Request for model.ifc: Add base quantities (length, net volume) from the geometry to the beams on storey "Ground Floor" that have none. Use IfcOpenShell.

First a look at what the model holds.

```python
import ifcopenshell
import ifcopenshell.util.element
import ifcopenshell.util.unit

model = ifcopenshell.open("model.ifc")
print(model.schema)
for unit_type in ("LENGTHUNIT", "AREAUNIT", "VOLUMEUNIT"):
    print(unit_type, ifcopenshell.util.unit.calculate_unit_scale(model, unit_type))
storey = next(s for s in model.by_type("IfcBuildingStorey") if s.Name == "Ground Floor")
beams = [e for e in ifcopenshell.util.element.get_decomposition(storey) if e.is_a("IfcBeam")]
for e in sorted(beams, key=lambda e: e.id()):
    print(e.id(), e.is_a(), e.Name, list(ifcopenshell.util.element.get_psets(e, qtos_only=True)), sep=" | ")
```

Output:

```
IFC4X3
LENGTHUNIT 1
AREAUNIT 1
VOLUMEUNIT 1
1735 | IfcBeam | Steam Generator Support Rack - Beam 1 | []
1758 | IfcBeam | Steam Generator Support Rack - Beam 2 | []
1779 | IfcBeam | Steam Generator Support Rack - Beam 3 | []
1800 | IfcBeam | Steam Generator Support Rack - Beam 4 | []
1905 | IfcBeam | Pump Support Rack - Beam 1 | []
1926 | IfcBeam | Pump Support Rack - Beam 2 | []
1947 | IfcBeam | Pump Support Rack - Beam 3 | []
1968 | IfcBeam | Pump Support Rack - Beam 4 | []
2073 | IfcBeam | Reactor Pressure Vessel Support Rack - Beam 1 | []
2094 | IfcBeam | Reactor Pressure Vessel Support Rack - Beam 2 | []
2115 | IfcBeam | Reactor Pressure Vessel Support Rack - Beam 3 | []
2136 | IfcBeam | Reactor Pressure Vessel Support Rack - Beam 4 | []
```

```python
import ifcopenshell
import ifcopenshell.api.pset
import ifcopenshell.geom
import ifcopenshell.util.element
import ifcopenshell.util.shape
import ifcopenshell.util.unit

model = ifcopenshell.open("model.ifc")
unit_scale = ifcopenshell.util.unit.calculate_unit_scale(model)
volume_scale = ifcopenshell.util.unit.calculate_unit_scale(model, "VOLUMEUNIT")
settings = ifcopenshell.geom.settings()

storey = next(s for s in model.by_type("IfcBuildingStorey") if s.Name == "Ground Floor")
beams = [e for e in ifcopenshell.util.element.get_decomposition(storey) if e.is_a("IfcBeam")]

for e in sorted(beams, key=lambda e: e.id()):
    if ifcopenshell.util.element.get_psets(e, qtos_only=True, should_inherit=False):
        continue
    # Geometry comes back in metres, in the element's own axes.
    shape = ifcopenshell.geom.create_shape(settings, e)
    values = {
        "Length": ifcopenshell.util.shape.get_max_xyz(shape.geometry) / unit_scale,
        "NetVolume": ifcopenshell.util.shape.get_volume(shape.geometry) / volume_scale,
    }
    qto = ifcopenshell.api.pset.add_qto(model, product=e, name="Qto_BeamBaseQuantities")
    ifcopenshell.api.pset.edit_qto(model, qto=qto, properties=values)
    print(e.id(), {k: round(v, 3) for k, v in values.items()})

model.write("model_edited.ifc")
```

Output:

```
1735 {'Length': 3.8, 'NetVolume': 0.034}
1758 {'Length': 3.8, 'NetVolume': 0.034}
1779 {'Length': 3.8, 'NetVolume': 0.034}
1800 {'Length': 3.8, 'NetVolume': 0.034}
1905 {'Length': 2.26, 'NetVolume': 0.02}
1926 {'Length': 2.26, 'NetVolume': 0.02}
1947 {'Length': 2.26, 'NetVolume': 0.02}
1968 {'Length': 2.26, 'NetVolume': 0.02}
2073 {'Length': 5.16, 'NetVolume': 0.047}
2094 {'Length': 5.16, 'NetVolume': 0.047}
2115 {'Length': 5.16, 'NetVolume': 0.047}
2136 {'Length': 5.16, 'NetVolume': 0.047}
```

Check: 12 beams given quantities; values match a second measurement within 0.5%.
